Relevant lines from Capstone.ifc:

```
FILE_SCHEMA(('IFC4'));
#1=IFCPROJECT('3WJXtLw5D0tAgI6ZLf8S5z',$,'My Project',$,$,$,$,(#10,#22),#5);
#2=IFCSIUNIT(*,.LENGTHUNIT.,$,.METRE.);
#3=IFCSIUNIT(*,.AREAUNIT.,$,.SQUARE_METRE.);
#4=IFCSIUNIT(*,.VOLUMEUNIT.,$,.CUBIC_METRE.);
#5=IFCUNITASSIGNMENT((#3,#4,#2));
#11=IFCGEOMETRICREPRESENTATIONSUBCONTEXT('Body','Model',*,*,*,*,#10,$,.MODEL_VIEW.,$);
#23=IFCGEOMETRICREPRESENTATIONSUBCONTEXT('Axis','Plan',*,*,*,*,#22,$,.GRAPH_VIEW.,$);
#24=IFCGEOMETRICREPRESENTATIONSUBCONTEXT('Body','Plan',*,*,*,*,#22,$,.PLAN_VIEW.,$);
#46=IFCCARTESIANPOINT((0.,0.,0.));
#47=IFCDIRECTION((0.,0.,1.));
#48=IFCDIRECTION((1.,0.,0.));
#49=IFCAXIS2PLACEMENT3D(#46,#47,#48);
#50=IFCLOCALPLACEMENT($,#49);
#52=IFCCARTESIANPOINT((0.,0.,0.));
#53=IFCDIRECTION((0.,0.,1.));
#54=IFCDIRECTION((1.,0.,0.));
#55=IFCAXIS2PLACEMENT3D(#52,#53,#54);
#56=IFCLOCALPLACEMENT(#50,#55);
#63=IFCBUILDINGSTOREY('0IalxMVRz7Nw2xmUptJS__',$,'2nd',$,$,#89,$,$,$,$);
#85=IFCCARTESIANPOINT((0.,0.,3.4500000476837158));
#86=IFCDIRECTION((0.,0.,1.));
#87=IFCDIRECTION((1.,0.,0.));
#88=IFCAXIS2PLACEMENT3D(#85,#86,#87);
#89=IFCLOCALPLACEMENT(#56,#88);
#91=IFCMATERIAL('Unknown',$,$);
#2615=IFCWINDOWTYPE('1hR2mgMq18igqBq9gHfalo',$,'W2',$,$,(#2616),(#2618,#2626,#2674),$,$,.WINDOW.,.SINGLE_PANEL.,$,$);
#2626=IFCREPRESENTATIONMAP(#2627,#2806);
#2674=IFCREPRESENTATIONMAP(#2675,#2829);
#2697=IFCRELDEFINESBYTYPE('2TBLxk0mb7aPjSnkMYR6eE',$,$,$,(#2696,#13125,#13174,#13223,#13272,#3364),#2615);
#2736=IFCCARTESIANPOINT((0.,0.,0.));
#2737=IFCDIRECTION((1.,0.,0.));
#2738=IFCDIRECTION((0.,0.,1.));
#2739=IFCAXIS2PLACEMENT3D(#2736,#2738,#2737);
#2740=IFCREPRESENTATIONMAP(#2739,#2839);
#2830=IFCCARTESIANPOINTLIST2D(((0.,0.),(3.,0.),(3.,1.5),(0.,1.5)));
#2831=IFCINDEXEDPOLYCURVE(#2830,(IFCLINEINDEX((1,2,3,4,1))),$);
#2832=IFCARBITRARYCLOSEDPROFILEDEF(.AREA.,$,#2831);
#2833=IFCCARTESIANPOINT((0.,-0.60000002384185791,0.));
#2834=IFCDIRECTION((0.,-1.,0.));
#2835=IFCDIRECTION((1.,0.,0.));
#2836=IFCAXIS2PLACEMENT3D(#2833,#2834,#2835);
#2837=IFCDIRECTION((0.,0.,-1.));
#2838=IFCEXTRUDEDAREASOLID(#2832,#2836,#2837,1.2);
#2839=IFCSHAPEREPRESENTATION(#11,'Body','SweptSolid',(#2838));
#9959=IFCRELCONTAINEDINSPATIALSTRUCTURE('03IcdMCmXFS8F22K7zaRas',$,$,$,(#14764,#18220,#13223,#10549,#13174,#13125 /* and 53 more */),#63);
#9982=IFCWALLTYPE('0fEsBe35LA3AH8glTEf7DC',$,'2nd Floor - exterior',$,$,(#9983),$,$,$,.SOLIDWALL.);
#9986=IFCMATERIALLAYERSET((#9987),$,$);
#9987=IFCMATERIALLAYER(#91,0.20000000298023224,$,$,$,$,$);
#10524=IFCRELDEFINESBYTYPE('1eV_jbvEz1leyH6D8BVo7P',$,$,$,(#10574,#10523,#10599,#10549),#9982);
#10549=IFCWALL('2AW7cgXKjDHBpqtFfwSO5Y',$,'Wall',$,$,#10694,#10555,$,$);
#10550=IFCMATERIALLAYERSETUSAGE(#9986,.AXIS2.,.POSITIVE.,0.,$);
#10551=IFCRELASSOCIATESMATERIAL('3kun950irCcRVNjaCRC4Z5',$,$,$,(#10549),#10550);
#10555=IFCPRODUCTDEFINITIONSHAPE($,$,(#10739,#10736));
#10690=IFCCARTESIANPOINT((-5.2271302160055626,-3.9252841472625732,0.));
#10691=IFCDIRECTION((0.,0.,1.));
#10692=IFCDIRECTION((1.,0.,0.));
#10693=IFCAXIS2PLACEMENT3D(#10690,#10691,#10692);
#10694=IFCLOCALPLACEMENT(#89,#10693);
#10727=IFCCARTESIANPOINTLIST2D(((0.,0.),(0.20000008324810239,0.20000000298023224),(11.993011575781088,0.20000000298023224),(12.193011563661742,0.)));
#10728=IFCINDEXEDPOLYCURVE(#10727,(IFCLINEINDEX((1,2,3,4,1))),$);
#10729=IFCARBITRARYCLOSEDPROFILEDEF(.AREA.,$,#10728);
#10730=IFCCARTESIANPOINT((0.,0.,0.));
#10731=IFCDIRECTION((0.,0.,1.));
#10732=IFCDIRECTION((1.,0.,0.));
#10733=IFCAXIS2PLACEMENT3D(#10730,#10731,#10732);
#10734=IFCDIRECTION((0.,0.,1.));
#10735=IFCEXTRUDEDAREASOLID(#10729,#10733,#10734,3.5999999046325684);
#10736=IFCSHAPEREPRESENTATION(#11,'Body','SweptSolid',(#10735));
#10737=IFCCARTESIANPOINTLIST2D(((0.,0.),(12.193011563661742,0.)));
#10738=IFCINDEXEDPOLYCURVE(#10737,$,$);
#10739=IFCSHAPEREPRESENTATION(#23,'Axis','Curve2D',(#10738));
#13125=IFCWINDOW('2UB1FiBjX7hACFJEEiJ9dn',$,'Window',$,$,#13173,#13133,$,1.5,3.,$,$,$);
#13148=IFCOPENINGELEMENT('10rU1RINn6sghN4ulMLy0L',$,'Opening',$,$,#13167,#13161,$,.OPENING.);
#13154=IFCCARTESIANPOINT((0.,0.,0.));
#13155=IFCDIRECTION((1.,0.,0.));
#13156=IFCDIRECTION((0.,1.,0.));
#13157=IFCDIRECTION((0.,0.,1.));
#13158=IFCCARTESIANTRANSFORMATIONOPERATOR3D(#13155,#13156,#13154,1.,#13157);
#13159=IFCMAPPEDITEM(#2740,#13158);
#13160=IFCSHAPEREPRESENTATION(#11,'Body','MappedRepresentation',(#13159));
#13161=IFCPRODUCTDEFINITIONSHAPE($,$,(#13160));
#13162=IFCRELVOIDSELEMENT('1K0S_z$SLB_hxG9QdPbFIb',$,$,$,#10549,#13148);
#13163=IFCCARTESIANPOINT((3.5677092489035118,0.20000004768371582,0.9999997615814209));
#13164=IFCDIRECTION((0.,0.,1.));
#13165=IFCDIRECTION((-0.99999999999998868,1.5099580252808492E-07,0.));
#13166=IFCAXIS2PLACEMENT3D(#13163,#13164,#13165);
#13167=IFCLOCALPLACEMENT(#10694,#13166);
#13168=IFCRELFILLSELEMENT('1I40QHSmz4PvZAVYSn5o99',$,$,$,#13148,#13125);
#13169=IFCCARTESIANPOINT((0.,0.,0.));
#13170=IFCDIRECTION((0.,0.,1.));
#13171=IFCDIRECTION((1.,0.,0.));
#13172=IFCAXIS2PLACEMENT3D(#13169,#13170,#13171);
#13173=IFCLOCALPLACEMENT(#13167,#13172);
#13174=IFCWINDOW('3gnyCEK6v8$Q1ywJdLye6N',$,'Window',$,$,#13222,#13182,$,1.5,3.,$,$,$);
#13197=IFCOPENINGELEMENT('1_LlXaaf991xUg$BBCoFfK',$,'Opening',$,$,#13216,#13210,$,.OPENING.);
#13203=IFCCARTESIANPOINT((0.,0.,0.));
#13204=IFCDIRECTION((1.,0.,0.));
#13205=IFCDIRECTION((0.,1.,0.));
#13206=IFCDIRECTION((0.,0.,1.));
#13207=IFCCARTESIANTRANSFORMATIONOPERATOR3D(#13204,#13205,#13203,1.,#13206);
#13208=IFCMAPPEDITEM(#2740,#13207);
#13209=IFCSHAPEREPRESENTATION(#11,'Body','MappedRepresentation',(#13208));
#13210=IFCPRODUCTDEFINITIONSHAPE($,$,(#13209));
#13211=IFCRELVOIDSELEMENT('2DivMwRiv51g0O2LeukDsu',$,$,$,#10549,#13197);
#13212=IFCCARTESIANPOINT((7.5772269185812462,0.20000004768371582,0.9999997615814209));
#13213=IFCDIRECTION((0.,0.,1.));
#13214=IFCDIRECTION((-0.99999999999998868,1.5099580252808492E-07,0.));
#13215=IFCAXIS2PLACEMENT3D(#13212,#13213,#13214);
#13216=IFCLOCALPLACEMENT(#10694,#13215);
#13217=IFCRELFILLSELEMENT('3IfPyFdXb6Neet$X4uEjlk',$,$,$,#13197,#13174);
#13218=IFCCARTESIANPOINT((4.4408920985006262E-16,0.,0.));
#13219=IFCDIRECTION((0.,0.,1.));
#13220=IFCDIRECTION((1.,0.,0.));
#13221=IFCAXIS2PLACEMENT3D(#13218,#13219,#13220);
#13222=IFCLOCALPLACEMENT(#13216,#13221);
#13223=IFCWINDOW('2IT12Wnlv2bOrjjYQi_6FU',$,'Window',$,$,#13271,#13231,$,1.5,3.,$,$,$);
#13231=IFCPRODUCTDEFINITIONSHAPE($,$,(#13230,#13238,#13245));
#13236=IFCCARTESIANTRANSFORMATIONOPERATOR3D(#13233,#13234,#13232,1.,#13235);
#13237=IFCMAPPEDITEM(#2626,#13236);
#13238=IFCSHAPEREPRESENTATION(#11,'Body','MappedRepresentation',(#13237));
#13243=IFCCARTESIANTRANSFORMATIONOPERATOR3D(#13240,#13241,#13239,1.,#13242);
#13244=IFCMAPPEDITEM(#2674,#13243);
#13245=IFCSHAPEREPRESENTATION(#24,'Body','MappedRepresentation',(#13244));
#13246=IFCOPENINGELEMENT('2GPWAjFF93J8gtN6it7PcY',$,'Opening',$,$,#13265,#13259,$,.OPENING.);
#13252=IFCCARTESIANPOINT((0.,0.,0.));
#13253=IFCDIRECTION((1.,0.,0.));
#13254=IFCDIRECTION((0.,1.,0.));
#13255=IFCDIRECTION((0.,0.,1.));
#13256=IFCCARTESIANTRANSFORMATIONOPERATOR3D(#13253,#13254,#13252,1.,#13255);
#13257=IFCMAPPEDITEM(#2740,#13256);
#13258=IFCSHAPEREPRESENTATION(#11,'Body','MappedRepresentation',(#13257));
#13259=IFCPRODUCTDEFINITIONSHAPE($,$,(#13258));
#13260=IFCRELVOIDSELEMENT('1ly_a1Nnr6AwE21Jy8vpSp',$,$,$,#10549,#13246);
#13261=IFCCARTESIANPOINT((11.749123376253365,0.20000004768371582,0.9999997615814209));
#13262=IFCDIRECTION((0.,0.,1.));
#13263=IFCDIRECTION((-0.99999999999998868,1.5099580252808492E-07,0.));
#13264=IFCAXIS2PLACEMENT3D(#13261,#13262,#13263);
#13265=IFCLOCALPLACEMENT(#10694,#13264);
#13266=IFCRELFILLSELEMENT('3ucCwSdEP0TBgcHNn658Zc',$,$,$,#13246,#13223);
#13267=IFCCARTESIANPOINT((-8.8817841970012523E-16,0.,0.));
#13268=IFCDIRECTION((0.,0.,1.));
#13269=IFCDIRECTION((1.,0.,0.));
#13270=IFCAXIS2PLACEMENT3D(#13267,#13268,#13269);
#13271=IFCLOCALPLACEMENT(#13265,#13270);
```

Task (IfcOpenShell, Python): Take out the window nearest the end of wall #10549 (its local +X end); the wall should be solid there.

```python
import ifcopenshell
import ifcopenshell.api.feature
import ifcopenshell.api.root
import ifcopenshell.geom
import ifcopenshell.util.shape

model = ifcopenshell.open("Capstone.ifc")
settings = ifcopenshell.geom.settings()


def volume(element):
    """Net volume in cubic metres, openings subtracted."""
    shape = ifcopenshell.geom.create_shape(settings, element)
    return ifcopenshell.util.shape.get_volume(shape.geometry)


window = model.by_guid("2IT12Wnlv2bOrjjYQi_6FU")
opening = window.FillsVoids[0].RelatingOpeningElement
wall = opening.VoidsElements[0].RelatingBuildingElement
before = volume(wall)

ifcopenshell.api.root.remove_product(model, product=window)
ifcopenshell.api.feature.remove_feature(model, feature=opening)

after = volume(wall)

print(f"wall volume {before:.3f} -> {after:.3f} m3")

model.write("Capstone-out.ifc")
```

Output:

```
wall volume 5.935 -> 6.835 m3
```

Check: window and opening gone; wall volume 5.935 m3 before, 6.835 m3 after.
